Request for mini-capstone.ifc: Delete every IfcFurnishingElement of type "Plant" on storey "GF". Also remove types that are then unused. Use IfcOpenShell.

First a look at what the model holds.

```python
import ifcopenshell
import ifcopenshell.util.element

model = ifcopenshell.open("mini-capstone.ifc")
print(model.schema)
storey = next(s for s in model.by_type("IfcBuildingStorey") if s.Name == "GF")
furniture = [e for e in ifcopenshell.util.element.get_decomposition(storey) if e.is_a("IfcFurnishingElement")]
seen = {}
for e in furniture:
    element_type = ifcopenshell.util.element.get_type(e)
    name = element_type.Name if element_type not in (None, e) else None
    seen[name] = seen.get(name, 0) + 1
for name, count in sorted(seen.items(), key=str):
    print(count, "x", name)
```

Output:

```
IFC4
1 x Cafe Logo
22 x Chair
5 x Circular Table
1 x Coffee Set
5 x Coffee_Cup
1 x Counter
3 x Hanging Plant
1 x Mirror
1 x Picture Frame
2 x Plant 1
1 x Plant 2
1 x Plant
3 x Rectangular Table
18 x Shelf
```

```python
import ifcopenshell
import ifcopenshell.api.root
import ifcopenshell.util.element

model = ifcopenshell.open("mini-capstone.ifc")

storey = next(s for s in model.by_type("IfcBuildingStorey") if s.Name == "GF")
furniture = [e for e in ifcopenshell.util.element.get_decomposition(storey) if e.is_a("IfcFurnishingElement")]
targets = [e for e in furniture if (t := ifcopenshell.util.element.get_type(e)) not in (None, e) and t.Name == "Plant"]
types = {ifcopenshell.util.element.get_type(e) for e in targets} - {None, *targets}

for e in targets:
    ifcopenshell.api.root.remove_product(model, product=e)
print(len(targets), "removed")

unused = [t for t in types if not ifcopenshell.util.element.get_types(t)]
for t in unused:
    ifcopenshell.api.root.remove_product(model, product=t)
print(len(unused), "unused types removed")

model.write("mini-capstone_updated.ifc")
```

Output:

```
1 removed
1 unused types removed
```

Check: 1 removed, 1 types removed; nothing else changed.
